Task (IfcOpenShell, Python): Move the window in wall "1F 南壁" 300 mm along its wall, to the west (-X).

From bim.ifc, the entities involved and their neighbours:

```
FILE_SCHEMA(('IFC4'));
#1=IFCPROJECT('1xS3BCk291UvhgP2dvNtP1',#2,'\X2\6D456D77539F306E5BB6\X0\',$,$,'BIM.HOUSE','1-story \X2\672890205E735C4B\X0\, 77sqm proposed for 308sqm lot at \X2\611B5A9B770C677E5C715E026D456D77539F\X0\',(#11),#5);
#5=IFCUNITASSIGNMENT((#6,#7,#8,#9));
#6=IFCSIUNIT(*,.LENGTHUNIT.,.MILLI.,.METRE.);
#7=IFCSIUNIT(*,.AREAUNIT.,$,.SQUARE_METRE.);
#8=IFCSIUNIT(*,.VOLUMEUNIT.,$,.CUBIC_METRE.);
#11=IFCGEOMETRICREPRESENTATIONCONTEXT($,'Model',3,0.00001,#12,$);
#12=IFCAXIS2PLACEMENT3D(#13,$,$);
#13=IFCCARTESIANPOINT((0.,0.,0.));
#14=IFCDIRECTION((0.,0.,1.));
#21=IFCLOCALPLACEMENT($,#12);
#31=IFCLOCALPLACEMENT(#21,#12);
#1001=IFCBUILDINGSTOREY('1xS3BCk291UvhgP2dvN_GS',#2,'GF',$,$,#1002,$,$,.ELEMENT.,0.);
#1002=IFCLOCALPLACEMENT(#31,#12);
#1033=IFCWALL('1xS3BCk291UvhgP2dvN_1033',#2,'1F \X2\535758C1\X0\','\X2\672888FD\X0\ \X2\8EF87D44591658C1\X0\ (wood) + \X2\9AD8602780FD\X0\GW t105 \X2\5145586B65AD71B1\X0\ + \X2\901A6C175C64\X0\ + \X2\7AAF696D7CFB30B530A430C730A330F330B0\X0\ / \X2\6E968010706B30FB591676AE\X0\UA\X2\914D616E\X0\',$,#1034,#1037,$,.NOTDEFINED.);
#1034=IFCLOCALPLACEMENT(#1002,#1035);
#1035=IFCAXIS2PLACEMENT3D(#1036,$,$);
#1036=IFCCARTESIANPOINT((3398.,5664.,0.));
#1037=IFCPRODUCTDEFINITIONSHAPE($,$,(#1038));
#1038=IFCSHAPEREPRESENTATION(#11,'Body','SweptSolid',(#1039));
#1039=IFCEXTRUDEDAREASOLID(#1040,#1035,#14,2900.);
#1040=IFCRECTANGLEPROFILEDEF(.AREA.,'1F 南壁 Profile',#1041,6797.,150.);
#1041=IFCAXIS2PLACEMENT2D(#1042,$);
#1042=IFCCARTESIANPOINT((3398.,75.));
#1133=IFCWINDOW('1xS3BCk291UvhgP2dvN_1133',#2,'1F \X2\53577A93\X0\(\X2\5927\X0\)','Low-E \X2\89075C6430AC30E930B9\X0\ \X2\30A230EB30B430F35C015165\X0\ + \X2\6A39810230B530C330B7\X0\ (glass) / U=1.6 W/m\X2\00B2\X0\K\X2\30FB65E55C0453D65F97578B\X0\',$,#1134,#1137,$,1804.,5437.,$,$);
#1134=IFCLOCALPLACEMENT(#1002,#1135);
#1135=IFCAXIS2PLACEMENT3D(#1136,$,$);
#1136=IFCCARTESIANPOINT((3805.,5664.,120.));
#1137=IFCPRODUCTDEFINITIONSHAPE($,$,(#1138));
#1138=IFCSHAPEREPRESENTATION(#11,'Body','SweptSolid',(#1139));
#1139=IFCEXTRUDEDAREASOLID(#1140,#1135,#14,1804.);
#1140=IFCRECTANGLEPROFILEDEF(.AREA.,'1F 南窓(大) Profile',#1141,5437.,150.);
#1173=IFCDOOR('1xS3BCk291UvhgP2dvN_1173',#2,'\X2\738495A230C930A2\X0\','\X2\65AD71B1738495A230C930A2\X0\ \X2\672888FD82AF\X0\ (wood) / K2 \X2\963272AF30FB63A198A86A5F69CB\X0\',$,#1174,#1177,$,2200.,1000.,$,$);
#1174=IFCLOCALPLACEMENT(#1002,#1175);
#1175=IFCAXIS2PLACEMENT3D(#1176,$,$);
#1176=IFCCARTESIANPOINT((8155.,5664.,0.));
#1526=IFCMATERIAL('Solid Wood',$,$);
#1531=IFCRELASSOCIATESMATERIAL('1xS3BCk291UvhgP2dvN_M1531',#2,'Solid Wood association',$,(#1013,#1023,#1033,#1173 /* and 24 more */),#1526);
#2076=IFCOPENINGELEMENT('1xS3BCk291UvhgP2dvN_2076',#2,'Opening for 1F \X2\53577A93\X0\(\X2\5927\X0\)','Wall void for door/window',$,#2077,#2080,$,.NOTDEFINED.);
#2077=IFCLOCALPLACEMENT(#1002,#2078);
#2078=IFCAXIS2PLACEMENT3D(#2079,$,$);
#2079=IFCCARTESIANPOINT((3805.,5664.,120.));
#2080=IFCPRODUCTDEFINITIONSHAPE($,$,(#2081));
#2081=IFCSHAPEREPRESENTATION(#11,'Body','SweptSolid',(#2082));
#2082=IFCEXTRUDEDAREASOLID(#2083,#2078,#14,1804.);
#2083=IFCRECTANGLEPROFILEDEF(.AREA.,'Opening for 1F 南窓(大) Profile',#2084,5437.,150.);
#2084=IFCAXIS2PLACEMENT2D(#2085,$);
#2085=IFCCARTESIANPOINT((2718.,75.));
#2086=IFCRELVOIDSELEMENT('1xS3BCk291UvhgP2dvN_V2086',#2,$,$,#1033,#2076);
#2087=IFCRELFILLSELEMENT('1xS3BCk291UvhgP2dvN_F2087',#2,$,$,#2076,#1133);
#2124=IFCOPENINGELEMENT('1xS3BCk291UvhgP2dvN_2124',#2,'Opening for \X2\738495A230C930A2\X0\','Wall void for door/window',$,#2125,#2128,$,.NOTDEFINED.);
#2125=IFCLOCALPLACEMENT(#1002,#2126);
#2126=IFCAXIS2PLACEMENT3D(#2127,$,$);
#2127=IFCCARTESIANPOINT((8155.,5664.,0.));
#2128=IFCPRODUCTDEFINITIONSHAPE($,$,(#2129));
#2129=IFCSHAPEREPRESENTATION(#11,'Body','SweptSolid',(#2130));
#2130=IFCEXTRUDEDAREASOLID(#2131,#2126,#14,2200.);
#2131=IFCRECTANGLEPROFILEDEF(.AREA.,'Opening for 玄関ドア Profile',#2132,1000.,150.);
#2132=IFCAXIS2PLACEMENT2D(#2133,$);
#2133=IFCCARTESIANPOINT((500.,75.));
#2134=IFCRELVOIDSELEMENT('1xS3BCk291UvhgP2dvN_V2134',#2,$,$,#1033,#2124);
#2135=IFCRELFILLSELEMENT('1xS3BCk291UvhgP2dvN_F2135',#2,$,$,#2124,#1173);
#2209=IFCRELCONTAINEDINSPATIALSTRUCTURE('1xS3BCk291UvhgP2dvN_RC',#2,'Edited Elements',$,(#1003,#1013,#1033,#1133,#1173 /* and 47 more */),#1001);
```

```python
import ifcopenshell
import ifcopenshell.api.geometry
import ifcopenshell.util.placement
import ifcopenshell.util.unit

model = ifcopenshell.open("bim.ifc")
unit_scale = ifcopenshell.util.unit.calculate_unit_scale(model)

window = model.by_guid("1xS3BCk291UvhgP2dvN_1133")
opening = window.FillsVoids[0].RelatingOpeningElement
wall = opening.VoidsElements[0].RelatingBuildingElement

wall_matrix = ifcopenshell.util.placement.get_local_placement(wall.ObjectPlacement)
shift = wall_matrix[:3, 0] * -0.3 / unit_scale
before = ifcopenshell.util.placement.get_local_placement(window.ObjectPlacement)[:3, 3].copy()

# The window is not placed relative to its opening, so move both.
for product in (opening, window):
    matrix = ifcopenshell.util.placement.get_local_placement(product.ObjectPlacement)
    matrix[:3, 3] += shift
    ifcopenshell.api.geometry.edit_object_placement(model, product=product, matrix=matrix, is_si=False)

after = ifcopenshell.util.placement.get_local_placement(window.ObjectPlacement)[:3, 3]
print("window moved by", (after - before).round(3) + 0.0)

model.write("bim-out.ifc")
```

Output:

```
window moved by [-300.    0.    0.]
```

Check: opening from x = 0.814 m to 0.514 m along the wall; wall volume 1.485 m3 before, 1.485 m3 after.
